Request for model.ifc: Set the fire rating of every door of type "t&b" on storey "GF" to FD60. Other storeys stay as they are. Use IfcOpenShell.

First a look at what the model holds.

```python
import ifcopenshell
import ifcopenshell.util.element

model = ifcopenshell.open("model.ifc")
print(model.schema)
storey = next(s for s in model.by_type("IfcBuildingStorey") if s.Name == "GF")
doors = [e for e in ifcopenshell.util.element.get_decomposition(storey) if e.is_a("IfcDoor")]
seen = {}
for e in doors:
    element_type = ifcopenshell.util.element.get_type(e)
    key = (element_type.Name if element_type != e and element_type else None, ifcopenshell.util.element.get_pset(e, "Pset_DoorCommon", "FireRating"))
    seen[key] = seen.get(key, 0) + 1
for (name, value), count in sorted(seen.items(), key=str):
    print(count, "x", name, "|", value)
```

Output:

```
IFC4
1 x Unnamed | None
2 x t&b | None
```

```python
import ifcopenshell
import ifcopenshell.api.pset
import ifcopenshell.util.element

model = ifcopenshell.open("model.ifc")

storey = next(s for s in model.by_type("IfcBuildingStorey") if s.Name == "GF")
doors = [e for e in ifcopenshell.util.element.get_decomposition(storey) if e.is_a("IfcDoor")]

count = 0
for e in doors:
    element_type = ifcopenshell.util.element.get_type(e)
    if element_type in (None, e) or element_type.Name != "t&b":
        continue
    # add_pset returns the element's existing set when there is one.
    pset = ifcopenshell.api.pset.add_pset(model, product=e, name="Pset_DoorCommon")
    ifcopenshell.api.pset.edit_pset(model, pset=pset, properties={"FireRating": "FD60"})
    count += 1

print(count, "doors updated")

model.write("model-out.ifc")
```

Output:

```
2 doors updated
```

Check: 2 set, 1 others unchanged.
